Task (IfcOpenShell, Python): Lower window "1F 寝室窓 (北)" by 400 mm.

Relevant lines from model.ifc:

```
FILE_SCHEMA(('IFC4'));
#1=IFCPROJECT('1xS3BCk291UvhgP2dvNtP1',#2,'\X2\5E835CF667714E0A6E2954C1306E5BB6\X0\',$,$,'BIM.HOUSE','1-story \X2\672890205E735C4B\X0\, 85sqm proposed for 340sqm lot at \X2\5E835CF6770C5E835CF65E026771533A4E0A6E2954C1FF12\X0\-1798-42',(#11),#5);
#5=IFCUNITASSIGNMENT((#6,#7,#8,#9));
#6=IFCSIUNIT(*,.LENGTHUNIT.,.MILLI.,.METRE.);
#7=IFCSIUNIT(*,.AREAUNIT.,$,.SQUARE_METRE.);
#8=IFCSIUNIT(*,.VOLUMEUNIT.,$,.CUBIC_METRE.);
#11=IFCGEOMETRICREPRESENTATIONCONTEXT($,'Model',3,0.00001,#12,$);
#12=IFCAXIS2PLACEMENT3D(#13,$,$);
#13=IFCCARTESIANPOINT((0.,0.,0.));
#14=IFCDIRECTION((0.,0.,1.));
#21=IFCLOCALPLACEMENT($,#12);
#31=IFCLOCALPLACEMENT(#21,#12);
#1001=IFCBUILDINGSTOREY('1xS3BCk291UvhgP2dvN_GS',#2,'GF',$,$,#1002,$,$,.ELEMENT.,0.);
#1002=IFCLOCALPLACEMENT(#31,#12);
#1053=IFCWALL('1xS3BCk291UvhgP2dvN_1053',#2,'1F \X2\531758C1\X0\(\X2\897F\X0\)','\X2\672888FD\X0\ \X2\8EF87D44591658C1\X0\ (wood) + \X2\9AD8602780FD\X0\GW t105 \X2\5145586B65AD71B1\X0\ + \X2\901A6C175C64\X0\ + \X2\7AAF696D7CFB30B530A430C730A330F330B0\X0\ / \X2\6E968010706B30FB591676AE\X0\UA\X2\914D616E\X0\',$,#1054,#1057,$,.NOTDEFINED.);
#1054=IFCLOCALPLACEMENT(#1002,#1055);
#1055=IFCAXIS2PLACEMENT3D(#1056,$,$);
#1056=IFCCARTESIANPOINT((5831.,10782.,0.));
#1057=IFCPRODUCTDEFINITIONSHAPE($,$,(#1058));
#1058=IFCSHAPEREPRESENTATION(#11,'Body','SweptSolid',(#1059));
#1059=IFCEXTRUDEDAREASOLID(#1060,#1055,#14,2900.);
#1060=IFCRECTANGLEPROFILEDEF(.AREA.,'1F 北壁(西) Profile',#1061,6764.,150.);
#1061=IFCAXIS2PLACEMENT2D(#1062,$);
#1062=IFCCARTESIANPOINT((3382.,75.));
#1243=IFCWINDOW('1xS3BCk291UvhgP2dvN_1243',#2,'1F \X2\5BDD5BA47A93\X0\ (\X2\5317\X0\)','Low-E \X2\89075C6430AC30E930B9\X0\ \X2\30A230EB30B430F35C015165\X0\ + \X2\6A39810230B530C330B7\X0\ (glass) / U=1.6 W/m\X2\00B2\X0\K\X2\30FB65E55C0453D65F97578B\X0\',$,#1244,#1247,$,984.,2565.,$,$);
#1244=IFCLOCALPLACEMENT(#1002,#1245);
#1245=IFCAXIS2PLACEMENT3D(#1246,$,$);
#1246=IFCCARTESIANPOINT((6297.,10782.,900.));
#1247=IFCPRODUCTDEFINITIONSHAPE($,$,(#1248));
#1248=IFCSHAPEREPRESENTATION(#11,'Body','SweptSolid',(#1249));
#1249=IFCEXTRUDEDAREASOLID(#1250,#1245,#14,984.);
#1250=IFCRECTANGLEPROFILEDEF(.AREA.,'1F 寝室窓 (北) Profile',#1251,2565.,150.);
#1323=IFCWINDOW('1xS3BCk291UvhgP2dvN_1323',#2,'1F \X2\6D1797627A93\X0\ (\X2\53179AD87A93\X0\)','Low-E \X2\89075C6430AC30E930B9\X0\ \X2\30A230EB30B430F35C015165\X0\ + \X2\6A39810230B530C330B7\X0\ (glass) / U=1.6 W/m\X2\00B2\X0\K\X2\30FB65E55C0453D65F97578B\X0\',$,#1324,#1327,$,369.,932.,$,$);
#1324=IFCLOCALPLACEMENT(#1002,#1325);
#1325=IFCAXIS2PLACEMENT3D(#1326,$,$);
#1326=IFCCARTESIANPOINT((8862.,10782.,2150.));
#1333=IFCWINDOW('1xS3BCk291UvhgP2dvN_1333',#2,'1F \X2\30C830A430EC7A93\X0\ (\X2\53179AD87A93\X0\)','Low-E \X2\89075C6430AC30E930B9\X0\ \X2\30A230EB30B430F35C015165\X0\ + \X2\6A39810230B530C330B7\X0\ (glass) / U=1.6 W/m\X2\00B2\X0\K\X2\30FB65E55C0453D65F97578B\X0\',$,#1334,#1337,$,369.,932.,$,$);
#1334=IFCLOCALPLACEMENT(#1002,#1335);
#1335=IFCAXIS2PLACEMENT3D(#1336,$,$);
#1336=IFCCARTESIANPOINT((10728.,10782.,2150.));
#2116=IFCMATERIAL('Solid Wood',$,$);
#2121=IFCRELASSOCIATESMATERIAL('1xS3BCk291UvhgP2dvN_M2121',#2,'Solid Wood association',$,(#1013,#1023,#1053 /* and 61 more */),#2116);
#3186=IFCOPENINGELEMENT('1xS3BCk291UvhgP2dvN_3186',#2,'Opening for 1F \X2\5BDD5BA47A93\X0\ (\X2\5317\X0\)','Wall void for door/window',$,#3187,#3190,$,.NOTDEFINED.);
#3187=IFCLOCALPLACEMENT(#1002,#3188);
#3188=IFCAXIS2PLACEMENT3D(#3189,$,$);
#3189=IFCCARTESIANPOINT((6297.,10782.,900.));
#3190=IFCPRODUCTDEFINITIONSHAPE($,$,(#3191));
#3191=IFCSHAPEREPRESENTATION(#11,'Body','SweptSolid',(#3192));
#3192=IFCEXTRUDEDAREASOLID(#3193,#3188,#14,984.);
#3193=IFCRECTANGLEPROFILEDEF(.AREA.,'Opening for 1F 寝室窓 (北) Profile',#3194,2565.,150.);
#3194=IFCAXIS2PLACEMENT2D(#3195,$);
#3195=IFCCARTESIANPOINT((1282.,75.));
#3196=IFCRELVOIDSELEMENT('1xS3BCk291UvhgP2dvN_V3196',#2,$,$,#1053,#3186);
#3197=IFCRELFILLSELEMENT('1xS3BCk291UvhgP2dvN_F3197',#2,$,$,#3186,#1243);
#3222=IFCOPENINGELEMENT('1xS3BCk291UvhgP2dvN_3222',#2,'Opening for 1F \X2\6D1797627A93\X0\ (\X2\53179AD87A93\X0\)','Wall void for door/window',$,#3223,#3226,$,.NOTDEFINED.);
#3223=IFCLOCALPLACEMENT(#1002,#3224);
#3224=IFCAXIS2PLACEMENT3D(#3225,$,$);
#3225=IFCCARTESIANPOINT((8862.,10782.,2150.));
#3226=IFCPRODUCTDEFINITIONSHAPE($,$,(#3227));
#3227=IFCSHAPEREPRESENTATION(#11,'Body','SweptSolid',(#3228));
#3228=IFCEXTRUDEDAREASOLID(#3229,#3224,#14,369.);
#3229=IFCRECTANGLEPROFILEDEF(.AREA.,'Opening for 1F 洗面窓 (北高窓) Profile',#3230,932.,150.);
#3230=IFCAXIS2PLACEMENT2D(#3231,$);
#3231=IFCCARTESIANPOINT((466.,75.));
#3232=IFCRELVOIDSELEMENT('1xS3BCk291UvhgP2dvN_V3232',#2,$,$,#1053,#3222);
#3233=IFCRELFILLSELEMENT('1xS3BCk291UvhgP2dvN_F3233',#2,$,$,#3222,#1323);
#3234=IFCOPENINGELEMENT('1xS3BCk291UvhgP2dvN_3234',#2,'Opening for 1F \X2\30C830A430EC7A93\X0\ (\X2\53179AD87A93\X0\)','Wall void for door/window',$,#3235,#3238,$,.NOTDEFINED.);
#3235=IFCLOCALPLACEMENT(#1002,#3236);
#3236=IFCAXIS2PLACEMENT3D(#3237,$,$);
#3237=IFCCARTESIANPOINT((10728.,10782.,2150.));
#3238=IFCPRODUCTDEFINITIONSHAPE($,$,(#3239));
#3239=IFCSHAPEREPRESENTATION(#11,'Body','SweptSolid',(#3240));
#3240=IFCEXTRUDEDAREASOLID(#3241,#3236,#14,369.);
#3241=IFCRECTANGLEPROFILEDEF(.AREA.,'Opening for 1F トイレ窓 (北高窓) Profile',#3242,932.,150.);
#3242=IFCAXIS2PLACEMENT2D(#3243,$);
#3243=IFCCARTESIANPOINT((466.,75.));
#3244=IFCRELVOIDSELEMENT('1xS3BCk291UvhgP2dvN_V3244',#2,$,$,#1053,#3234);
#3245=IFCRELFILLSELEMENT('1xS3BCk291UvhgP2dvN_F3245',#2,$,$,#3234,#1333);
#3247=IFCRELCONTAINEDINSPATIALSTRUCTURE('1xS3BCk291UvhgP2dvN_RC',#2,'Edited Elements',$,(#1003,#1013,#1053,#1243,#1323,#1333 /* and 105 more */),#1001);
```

```python
import numpy as np
import ifcopenshell
import ifcopenshell.api.geometry
import ifcopenshell.util.placement
import ifcopenshell.util.unit

model = ifcopenshell.open("model.ifc")
unit_scale = ifcopenshell.util.unit.calculate_unit_scale(model)

window = model.by_guid("1xS3BCk291UvhgP2dvN_1243")
opening = window.FillsVoids[0].RelatingOpeningElement
dz = -0.4 / unit_scale

shift = np.array([0.0, 0.0, dz])
# The window is not placed relative to its opening, so move both.
for product in (opening, window):
    matrix = ifcopenshell.util.placement.get_local_placement(product.ObjectPlacement)
    matrix[:3, 3] += shift
    ifcopenshell.api.geometry.edit_object_placement(model, product=product, matrix=matrix, is_si=False)

print(f"moved by {dz * unit_scale:+.3f} m")

model.write("model-out.ifc")
```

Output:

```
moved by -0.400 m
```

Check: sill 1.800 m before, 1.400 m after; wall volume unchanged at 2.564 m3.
